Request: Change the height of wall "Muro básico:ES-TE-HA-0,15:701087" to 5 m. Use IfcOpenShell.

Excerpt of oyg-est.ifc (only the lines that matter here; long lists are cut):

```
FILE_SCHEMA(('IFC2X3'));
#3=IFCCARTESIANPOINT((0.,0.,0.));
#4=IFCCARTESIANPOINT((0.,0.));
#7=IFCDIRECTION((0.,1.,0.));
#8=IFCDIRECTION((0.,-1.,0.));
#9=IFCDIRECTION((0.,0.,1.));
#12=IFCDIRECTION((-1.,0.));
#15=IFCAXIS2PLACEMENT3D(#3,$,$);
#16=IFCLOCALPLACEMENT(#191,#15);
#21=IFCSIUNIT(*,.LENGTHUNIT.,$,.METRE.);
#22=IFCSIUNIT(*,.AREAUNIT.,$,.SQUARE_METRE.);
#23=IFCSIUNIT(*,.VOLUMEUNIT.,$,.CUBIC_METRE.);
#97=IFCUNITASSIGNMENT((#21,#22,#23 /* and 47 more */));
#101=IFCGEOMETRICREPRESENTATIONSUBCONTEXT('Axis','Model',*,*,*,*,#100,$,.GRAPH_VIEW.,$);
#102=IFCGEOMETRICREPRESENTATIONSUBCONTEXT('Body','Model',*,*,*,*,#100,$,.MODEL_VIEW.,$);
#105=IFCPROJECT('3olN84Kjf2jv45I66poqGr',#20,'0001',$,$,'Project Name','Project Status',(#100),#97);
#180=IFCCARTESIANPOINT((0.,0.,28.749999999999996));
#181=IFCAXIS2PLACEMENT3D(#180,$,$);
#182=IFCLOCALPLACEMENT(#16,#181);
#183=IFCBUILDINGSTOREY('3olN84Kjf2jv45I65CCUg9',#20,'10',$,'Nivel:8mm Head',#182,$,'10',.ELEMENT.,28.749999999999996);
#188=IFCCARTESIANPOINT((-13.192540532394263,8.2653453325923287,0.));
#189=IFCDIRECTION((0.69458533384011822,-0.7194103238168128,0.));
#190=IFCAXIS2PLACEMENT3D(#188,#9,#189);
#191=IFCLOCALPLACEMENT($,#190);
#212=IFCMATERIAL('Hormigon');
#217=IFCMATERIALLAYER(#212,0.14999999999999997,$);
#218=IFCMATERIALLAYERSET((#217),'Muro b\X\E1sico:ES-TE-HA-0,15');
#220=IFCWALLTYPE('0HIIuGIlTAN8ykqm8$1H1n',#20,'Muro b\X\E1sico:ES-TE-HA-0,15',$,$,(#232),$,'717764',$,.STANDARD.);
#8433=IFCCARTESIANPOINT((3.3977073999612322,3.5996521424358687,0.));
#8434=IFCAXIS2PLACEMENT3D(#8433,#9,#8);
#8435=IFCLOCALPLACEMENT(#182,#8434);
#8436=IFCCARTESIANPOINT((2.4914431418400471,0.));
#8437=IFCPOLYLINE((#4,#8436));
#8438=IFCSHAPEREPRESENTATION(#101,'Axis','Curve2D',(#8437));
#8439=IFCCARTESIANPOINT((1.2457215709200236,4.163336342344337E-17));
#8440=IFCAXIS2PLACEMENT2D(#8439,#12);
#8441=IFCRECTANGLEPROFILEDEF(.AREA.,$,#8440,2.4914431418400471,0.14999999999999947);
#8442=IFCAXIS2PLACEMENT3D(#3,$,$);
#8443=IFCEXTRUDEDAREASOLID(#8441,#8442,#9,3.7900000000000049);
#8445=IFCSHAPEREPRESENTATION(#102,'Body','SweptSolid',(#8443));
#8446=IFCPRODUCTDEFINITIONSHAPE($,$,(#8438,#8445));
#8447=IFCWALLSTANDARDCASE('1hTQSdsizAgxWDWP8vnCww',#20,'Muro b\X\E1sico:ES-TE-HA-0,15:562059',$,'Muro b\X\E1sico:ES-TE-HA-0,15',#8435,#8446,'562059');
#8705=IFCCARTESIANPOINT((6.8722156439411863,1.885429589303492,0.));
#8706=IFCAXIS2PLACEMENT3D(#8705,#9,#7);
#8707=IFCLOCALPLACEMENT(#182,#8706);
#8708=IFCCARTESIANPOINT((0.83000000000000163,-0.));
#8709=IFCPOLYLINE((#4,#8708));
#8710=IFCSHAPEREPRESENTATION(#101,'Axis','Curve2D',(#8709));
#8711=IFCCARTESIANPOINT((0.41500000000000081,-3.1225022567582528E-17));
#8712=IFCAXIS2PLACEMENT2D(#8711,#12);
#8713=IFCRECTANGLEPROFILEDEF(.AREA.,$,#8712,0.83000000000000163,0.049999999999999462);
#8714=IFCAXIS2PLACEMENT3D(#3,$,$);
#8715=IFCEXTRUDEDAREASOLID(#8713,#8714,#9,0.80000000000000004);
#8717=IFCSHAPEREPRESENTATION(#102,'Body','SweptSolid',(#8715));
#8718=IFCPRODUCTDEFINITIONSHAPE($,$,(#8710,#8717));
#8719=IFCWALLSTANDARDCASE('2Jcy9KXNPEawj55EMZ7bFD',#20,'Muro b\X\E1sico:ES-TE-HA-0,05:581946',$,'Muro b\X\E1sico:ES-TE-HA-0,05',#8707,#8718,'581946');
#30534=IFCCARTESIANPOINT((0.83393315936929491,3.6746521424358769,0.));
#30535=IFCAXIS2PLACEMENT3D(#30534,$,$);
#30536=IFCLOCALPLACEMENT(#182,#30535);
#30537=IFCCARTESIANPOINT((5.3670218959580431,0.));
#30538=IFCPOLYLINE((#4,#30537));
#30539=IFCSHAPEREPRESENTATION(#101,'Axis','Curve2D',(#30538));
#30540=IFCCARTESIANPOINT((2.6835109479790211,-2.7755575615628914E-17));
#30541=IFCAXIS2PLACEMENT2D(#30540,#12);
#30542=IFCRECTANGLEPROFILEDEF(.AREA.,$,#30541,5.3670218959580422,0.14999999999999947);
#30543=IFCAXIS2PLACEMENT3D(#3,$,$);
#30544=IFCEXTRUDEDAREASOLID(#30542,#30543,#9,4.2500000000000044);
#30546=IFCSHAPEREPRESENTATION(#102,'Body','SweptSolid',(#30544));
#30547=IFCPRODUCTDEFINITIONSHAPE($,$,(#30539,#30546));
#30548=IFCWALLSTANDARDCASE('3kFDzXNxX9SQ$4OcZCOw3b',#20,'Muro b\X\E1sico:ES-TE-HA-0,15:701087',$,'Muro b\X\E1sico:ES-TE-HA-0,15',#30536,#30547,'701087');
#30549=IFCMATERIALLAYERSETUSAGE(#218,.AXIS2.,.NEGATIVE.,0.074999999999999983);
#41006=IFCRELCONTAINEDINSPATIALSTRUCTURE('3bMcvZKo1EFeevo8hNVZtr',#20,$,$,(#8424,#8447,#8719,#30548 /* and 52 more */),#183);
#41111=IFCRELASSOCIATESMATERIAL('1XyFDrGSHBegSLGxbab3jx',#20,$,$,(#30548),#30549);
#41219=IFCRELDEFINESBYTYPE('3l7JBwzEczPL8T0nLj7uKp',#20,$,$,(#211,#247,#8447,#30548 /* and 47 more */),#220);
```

```python
import ifcopenshell
import ifcopenshell.geom
import ifcopenshell.util.representation
import ifcopenshell.util.shape

model = ifcopenshell.open("oyg-est.ifc")
settings = ifcopenshell.geom.settings()


def volume(element):
    """Net volume in cubic metres, openings subtracted."""
    shape = ifcopenshell.geom.create_shape(settings, element)
    return ifcopenshell.util.shape.get_volume(shape.geometry)


wall = model.by_guid("3kFDzXNxX9SQ$4OcZCOw3b")
before = volume(wall)

body = ifcopenshell.util.representation.get_representation(wall, "Model", "Body")
solid = body.Items[0]
old_height = solid.Depth
solid.Depth = 5.0
after = volume(wall)

print(f"height {old_height:g} -> {solid.Depth:g}, volume {before:.3f} -> {after:.3f} m3")

model.write("oyg-est_rev.ifc")
```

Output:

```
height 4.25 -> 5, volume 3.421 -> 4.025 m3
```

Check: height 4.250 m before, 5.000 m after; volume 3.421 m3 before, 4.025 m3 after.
